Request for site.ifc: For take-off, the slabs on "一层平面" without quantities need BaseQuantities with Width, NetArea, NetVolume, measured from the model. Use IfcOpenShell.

First a look at what the model holds.

```python
import ifcopenshell
import ifcopenshell.util.element
import ifcopenshell.util.unit

model = ifcopenshell.open("site.ifc")
print(model.schema)
for unit_type in ("LENGTHUNIT", "AREAUNIT", "VOLUMEUNIT"):
    print(unit_type, ifcopenshell.util.unit.calculate_unit_scale(model, unit_type))
storey = next(s for s in model.by_type("IfcBuildingStorey") if s.Name == "一层平面")
slabs = [e for e in ifcopenshell.util.element.get_decomposition(storey) if e.is_a("IfcSlab")]
for e in sorted(slabs, key=lambda e: e.id()):
    print(e.id(), e.is_a(), e.Name, list(ifcopenshell.util.element.get_psets(e, qtos_only=True)), sep=" | ")
```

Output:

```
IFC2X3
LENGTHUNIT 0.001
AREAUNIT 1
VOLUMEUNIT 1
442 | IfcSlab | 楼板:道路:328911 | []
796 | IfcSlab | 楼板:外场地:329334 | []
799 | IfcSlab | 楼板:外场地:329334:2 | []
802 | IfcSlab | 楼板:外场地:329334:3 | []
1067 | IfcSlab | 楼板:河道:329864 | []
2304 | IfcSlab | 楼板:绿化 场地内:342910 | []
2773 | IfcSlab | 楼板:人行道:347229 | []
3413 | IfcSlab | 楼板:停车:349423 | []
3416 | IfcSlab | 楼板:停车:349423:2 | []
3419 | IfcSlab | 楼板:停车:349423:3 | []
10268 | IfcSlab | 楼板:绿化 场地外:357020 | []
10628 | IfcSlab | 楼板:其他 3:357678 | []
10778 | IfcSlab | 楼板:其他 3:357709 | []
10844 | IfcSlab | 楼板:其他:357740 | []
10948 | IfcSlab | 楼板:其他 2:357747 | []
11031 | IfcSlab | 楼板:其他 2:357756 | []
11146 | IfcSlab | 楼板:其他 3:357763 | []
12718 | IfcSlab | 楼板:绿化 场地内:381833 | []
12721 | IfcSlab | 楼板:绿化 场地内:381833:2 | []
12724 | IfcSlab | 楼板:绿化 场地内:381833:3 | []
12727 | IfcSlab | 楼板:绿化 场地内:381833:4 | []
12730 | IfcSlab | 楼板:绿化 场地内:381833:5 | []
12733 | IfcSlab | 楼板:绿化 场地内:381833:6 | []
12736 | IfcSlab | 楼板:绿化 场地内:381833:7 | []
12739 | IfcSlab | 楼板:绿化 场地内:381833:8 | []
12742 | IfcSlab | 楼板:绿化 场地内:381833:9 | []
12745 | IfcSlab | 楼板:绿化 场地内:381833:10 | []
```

```python
import ifcopenshell
import ifcopenshell.api.pset
import ifcopenshell.geom
import ifcopenshell.util.element
import ifcopenshell.util.shape
import ifcopenshell.util.unit

model = ifcopenshell.open("site.ifc")
unit_scale = ifcopenshell.util.unit.calculate_unit_scale(model)
area_scale = ifcopenshell.util.unit.calculate_unit_scale(model, "AREAUNIT")
volume_scale = ifcopenshell.util.unit.calculate_unit_scale(model, "VOLUMEUNIT")
settings = ifcopenshell.geom.settings()

storey = next(s for s in model.by_type("IfcBuildingStorey") if s.Name == "一层平面")
slabs = [e for e in ifcopenshell.util.element.get_decomposition(storey) if e.is_a("IfcSlab")]

for e in sorted(slabs, key=lambda e: e.id()):
    if ifcopenshell.util.element.get_psets(e, qtos_only=True, should_inherit=False):
        continue
    # Geometry comes back in metres, in the element's own axes.
    shape = ifcopenshell.geom.create_shape(settings, e)
    values = {
        "Width": ifcopenshell.util.shape.get_z(shape.geometry) / unit_scale,
        "NetArea": ifcopenshell.util.shape.get_footprint_area(shape.geometry) / area_scale,
        "NetVolume": ifcopenshell.util.shape.get_volume(shape.geometry) / volume_scale,
    }
    qto = ifcopenshell.api.pset.add_qto(model, product=e, name="BaseQuantities")
    ifcopenshell.api.pset.edit_qto(model, qto=qto, properties=values)
    print(e.id(), {k: round(v, 3) for k, v in values.items()})

model.write("site-out.ifc")
```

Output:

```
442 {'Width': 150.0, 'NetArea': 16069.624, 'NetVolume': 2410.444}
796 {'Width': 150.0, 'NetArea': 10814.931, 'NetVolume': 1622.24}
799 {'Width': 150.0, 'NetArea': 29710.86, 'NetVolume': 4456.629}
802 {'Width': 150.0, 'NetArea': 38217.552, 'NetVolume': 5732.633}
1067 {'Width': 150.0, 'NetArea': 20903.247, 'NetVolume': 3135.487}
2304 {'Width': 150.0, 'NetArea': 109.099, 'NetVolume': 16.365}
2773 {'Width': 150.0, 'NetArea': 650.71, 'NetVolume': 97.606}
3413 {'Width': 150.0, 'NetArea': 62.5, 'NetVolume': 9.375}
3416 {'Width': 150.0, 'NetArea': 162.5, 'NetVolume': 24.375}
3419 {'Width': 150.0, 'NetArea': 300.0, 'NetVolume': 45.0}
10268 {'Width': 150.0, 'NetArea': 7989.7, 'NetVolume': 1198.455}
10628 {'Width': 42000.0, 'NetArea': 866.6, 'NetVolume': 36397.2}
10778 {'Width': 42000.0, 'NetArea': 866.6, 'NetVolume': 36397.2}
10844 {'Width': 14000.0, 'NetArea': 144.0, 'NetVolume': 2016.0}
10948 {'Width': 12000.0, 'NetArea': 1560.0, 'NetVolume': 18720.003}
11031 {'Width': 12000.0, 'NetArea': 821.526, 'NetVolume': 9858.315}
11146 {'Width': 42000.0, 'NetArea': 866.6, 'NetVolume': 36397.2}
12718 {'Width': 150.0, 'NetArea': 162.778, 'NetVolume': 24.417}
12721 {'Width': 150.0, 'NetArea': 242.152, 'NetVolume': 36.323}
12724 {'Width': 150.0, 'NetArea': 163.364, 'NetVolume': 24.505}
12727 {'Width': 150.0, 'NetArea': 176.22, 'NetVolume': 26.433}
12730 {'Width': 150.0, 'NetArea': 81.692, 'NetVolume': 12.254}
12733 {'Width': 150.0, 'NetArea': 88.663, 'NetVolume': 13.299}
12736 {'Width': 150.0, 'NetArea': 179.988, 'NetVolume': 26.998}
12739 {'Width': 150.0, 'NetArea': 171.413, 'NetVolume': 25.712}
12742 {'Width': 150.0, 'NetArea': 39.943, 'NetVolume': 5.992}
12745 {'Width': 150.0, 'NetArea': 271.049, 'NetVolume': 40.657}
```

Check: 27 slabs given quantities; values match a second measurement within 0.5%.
